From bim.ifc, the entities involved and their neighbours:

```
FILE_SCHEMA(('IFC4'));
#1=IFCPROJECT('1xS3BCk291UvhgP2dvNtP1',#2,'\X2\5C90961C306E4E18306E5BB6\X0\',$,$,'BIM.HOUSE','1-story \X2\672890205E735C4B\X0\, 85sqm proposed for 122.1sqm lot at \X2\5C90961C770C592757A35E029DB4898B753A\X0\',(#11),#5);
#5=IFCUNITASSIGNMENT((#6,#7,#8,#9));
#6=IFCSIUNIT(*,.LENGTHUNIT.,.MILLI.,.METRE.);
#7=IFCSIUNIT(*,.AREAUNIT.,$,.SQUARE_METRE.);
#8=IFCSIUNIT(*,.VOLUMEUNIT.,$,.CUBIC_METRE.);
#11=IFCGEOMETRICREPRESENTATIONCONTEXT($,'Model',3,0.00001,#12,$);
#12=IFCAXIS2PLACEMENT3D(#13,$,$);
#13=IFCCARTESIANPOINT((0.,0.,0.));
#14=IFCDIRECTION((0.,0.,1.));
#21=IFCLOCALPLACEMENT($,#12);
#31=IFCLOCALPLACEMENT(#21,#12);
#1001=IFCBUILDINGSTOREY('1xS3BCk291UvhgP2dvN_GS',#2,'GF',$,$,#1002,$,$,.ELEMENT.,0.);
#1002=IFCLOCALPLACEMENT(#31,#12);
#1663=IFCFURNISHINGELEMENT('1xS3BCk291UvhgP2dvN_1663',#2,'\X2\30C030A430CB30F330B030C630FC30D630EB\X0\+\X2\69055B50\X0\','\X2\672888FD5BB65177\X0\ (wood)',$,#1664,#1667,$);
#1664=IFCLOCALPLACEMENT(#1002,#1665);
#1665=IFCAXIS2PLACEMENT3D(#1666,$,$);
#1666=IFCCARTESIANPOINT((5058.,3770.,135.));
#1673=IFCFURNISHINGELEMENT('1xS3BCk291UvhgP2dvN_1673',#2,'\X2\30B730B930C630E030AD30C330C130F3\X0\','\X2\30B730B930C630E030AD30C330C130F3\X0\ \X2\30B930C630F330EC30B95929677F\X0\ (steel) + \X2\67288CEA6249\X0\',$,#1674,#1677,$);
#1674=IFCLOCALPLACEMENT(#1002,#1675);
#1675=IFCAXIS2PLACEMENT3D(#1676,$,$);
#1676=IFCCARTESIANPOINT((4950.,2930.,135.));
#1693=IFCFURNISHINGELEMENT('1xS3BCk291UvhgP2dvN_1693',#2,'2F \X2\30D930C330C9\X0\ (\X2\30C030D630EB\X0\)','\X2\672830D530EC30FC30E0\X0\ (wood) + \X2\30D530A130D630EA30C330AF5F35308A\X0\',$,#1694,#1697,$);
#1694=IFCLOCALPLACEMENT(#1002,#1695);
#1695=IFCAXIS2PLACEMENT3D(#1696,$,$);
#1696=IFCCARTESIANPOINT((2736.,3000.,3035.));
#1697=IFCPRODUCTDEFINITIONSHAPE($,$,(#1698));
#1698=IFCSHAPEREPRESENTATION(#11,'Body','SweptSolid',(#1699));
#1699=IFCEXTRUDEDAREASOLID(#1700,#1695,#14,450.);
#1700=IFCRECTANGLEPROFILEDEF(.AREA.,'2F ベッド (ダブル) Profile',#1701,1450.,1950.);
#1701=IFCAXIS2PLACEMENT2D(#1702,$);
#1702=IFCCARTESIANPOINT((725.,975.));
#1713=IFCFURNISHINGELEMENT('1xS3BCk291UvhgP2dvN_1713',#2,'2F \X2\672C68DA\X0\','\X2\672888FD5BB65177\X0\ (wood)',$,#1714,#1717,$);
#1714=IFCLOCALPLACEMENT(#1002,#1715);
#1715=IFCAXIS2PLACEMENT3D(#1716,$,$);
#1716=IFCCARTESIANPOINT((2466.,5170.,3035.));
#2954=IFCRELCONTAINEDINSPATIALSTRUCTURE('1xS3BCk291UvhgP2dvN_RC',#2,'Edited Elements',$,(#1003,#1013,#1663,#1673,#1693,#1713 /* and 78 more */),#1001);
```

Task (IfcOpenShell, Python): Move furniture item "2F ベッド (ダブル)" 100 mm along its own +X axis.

```python
import ifcopenshell
import ifcopenshell.api.geometry
import ifcopenshell.util.placement

model = ifcopenshell.open("bim.ifc")

item = model.by_guid("1xS3BCk291UvhgP2dvN_1693")
matrix = ifcopenshell.util.placement.get_local_placement(item.ObjectPlacement)
matrix[:3, 3] += matrix[:3, 0] * 100.0
ifcopenshell.api.geometry.edit_object_placement(model, product=item, matrix=matrix, is_si=False)

print(ifcopenshell.util.placement.get_local_placement(item.ObjectPlacement).round(3) + 0.0)

model.write("bim_rev.ifc")
```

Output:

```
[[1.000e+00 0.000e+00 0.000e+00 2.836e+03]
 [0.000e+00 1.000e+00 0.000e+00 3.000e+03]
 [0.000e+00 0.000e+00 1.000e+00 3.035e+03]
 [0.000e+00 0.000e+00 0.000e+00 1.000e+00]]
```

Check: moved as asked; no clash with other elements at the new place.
